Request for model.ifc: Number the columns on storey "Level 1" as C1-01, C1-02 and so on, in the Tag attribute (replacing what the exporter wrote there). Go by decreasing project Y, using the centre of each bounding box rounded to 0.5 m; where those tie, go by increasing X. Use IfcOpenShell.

First a look at what the model holds.

```python
import ifcopenshell
import ifcopenshell.util.element
import ifcopenshell.util.placement

model = ifcopenshell.open("model.ifc")
print(model.schema)
storey = next(s for s in model.by_type("IfcBuildingStorey") if s.Name == "Level 1")
columns = [e for e in ifcopenshell.util.element.get_decomposition(storey) if e.is_a("IfcColumn")]
for e in sorted(columns, key=lambda e: e.id()):
    origin = ifcopenshell.util.placement.get_local_placement(e.ObjectPlacement)[:3, 3]
    print(e.id(), e.Tag, e.Name, origin.round(2) + 0.0, sep=" | ")
```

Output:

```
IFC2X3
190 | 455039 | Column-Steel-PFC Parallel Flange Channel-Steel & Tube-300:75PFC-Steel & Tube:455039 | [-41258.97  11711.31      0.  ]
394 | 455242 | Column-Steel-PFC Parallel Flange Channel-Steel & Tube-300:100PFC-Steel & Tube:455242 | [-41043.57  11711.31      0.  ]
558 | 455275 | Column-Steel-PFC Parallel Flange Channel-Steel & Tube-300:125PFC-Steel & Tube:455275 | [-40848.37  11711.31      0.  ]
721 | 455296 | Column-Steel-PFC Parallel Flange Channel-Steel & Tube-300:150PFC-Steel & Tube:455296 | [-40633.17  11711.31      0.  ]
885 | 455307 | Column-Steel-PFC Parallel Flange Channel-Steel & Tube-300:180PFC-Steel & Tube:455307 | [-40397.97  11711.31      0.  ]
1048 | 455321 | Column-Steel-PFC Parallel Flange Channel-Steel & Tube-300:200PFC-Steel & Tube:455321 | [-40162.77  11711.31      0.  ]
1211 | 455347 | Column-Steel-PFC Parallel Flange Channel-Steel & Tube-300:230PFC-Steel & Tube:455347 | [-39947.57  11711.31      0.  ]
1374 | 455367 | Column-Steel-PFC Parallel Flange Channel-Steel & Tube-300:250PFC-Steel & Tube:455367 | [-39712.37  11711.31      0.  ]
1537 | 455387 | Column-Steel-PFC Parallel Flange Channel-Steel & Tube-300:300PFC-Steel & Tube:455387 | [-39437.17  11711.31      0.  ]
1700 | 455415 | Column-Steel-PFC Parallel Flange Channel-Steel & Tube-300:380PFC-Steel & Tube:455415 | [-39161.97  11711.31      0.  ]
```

```python
import ifcopenshell
import ifcopenshell.geom
import ifcopenshell.util.element
import ifcopenshell.util.shape

model = ifcopenshell.open("model.ifc")
settings = ifcopenshell.geom.settings()
settings.set("use-world-coords", True)


def centre(element):
    shape = ifcopenshell.geom.create_shape(settings, element)
    return ifcopenshell.util.shape.get_bbox_centroid(shape.geometry)


storey = next(s for s in model.by_type("IfcBuildingStorey") if s.Name == "Level 1")
columns = [e for e in ifcopenshell.util.element.get_decomposition(storey) if e.is_a("IfcColumn")]

# Insertion points can sit at a corner or the storey origin, so sort by the geometry (in metres).
centres = {e: centre(e) for e in columns}
columns.sort(key=lambda e: (-round(centres[e][1] / 0.5), centres[e][0]))

for i, e in enumerate(columns, start=1):
    number = f"C1-{i:02d}"
    e.Tag = number
    print(e.id(), number)

model.write("model_updated.ifc")
```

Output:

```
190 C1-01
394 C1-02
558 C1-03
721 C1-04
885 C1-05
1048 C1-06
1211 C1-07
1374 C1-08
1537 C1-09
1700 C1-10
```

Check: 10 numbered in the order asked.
